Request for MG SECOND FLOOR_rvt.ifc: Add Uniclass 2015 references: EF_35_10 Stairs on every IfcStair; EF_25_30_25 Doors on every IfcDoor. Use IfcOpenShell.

First a look at what the model holds.

```python
import ifcopenshell

model = ifcopenshell.open("MG SECOND FLOOR_rvt.ifc")
print(model.schema)
print("classifications:", [c.Name for c in model.by_type("IfcClassification")])
for ifc_class in ("IfcDoor", "IfcRoof", "IfcStair", "IfcWall", "IfcWindow"):
    print(ifc_class, len(model.by_type(ifc_class)))
```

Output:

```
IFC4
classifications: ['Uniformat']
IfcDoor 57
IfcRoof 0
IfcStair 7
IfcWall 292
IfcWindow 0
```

```python
import ifcopenshell
import ifcopenshell.api.classification

model = ifcopenshell.open("MG SECOND FLOOR_rvt.ifc")

system = ifcopenshell.api.classification.add_classification(model, classification="Uniclass 2015")

codes = {
    "IfcStair": ("EF_35_10", "Stairs"),
    "IfcDoor": ("EF_25_30_25", "Doors"),
}
for ifc_class, (code, name) in codes.items():
    products = model.by_type(ifc_class)
    ifcopenshell.api.classification.add_reference(
        model, products=products, classification=system, identification=code, name=name
    )
    print(code, len(products))

model.write("MG SECOND FLOOR_rvt_rev.ifc")
```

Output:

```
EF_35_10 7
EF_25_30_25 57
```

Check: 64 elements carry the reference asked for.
